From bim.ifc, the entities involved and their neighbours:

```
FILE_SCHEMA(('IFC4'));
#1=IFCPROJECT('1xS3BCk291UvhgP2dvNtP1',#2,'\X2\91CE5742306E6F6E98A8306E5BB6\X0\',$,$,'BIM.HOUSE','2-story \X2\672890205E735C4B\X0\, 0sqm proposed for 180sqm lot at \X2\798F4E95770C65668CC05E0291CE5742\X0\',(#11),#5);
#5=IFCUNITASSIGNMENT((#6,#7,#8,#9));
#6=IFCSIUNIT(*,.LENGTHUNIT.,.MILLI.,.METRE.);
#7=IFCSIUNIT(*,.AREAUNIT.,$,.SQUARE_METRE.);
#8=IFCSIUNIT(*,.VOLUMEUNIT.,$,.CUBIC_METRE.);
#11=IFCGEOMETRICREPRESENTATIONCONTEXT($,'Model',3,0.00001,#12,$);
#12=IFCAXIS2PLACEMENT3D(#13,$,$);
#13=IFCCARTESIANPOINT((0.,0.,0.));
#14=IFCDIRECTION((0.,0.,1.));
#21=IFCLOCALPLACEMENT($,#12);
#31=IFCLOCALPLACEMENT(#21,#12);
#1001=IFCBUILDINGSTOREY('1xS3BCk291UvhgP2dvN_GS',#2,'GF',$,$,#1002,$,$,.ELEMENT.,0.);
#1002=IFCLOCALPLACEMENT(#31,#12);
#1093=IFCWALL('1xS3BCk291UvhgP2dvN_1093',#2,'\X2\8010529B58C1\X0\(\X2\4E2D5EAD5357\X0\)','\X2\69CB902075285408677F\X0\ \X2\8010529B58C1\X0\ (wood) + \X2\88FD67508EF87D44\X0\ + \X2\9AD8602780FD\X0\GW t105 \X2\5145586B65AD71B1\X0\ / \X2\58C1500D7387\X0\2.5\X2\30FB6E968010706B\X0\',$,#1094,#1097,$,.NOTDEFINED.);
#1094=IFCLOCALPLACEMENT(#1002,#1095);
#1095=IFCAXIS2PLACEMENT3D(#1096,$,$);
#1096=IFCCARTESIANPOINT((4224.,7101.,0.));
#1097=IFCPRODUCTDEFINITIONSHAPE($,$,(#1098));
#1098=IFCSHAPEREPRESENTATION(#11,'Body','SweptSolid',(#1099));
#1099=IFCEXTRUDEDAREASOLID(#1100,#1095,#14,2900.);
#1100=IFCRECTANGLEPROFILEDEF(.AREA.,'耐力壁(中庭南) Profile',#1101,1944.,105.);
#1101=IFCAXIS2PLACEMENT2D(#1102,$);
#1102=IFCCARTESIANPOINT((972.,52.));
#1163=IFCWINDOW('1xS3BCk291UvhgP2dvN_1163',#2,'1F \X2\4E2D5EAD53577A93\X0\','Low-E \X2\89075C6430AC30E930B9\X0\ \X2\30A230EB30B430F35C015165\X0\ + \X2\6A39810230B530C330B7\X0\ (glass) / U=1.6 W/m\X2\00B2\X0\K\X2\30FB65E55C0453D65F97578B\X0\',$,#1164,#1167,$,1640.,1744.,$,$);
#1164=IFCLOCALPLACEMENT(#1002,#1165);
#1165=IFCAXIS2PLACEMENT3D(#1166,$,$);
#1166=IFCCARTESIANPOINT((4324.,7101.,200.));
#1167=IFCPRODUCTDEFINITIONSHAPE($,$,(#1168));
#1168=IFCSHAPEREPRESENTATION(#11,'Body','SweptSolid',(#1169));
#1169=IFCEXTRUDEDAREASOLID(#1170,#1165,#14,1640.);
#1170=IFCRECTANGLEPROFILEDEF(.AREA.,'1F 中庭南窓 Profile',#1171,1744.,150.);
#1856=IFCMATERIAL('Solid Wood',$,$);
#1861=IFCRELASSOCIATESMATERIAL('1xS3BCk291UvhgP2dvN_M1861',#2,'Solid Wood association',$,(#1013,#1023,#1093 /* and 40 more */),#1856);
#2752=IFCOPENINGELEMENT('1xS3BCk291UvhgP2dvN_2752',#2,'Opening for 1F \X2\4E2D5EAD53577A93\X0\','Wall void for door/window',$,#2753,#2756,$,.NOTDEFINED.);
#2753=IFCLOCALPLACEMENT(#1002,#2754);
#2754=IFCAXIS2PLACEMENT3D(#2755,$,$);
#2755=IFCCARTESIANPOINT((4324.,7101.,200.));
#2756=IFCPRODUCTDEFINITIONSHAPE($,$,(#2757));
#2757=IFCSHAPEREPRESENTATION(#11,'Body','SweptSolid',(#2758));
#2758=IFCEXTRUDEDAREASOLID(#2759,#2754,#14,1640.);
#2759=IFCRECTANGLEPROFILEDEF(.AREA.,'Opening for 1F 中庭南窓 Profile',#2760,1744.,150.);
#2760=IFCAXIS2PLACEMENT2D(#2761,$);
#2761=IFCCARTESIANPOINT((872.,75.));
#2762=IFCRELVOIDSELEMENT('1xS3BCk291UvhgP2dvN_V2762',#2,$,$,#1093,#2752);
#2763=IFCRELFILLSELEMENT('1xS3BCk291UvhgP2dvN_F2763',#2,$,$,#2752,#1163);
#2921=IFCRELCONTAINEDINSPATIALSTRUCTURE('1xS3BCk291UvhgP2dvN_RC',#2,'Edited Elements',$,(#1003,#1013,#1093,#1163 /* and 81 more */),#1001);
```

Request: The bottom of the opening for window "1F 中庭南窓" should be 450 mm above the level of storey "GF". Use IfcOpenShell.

```python
import numpy as np
import ifcopenshell
import ifcopenshell.api.geometry
import ifcopenshell.geom
import ifcopenshell.util.element
import ifcopenshell.util.placement
import ifcopenshell.util.shape
import ifcopenshell.util.unit

model = ifcopenshell.open("bim.ifc")
unit_scale = ifcopenshell.util.unit.calculate_unit_scale(model)

window = model.by_guid("1xS3BCk291UvhgP2dvN_1163")
opening = window.FillsVoids[0].RelatingOpeningElement
storey = ifcopenshell.util.element.get_container(window, ifc_class="IfcBuildingStorey")
level = ifcopenshell.util.placement.get_local_placement(storey.ObjectPlacement)[2, 3]

# The opening's origin need not be at the sill, so measure its lowest point.
shape = ifcopenshell.geom.create_shape(ifcopenshell.geom.settings(), opening)
bottom = ifcopenshell.util.shape.get_shape_bottom_elevation(shape, shape.geometry) / unit_scale
dz = level + 450.0 - bottom

shift = np.array([0.0, 0.0, dz])
# The window is not placed relative to its opening, so move both.
for product in (opening, window):
    matrix = ifcopenshell.util.placement.get_local_placement(product.ObjectPlacement)
    matrix[:3, 3] += shift
    ifcopenshell.api.geometry.edit_object_placement(model, product=product, matrix=matrix, is_si=False)

print(f"moved by {dz * unit_scale:+.3f} m")

model.write("bim_updated.ifc")
```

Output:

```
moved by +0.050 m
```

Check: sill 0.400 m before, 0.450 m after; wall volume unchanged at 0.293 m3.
